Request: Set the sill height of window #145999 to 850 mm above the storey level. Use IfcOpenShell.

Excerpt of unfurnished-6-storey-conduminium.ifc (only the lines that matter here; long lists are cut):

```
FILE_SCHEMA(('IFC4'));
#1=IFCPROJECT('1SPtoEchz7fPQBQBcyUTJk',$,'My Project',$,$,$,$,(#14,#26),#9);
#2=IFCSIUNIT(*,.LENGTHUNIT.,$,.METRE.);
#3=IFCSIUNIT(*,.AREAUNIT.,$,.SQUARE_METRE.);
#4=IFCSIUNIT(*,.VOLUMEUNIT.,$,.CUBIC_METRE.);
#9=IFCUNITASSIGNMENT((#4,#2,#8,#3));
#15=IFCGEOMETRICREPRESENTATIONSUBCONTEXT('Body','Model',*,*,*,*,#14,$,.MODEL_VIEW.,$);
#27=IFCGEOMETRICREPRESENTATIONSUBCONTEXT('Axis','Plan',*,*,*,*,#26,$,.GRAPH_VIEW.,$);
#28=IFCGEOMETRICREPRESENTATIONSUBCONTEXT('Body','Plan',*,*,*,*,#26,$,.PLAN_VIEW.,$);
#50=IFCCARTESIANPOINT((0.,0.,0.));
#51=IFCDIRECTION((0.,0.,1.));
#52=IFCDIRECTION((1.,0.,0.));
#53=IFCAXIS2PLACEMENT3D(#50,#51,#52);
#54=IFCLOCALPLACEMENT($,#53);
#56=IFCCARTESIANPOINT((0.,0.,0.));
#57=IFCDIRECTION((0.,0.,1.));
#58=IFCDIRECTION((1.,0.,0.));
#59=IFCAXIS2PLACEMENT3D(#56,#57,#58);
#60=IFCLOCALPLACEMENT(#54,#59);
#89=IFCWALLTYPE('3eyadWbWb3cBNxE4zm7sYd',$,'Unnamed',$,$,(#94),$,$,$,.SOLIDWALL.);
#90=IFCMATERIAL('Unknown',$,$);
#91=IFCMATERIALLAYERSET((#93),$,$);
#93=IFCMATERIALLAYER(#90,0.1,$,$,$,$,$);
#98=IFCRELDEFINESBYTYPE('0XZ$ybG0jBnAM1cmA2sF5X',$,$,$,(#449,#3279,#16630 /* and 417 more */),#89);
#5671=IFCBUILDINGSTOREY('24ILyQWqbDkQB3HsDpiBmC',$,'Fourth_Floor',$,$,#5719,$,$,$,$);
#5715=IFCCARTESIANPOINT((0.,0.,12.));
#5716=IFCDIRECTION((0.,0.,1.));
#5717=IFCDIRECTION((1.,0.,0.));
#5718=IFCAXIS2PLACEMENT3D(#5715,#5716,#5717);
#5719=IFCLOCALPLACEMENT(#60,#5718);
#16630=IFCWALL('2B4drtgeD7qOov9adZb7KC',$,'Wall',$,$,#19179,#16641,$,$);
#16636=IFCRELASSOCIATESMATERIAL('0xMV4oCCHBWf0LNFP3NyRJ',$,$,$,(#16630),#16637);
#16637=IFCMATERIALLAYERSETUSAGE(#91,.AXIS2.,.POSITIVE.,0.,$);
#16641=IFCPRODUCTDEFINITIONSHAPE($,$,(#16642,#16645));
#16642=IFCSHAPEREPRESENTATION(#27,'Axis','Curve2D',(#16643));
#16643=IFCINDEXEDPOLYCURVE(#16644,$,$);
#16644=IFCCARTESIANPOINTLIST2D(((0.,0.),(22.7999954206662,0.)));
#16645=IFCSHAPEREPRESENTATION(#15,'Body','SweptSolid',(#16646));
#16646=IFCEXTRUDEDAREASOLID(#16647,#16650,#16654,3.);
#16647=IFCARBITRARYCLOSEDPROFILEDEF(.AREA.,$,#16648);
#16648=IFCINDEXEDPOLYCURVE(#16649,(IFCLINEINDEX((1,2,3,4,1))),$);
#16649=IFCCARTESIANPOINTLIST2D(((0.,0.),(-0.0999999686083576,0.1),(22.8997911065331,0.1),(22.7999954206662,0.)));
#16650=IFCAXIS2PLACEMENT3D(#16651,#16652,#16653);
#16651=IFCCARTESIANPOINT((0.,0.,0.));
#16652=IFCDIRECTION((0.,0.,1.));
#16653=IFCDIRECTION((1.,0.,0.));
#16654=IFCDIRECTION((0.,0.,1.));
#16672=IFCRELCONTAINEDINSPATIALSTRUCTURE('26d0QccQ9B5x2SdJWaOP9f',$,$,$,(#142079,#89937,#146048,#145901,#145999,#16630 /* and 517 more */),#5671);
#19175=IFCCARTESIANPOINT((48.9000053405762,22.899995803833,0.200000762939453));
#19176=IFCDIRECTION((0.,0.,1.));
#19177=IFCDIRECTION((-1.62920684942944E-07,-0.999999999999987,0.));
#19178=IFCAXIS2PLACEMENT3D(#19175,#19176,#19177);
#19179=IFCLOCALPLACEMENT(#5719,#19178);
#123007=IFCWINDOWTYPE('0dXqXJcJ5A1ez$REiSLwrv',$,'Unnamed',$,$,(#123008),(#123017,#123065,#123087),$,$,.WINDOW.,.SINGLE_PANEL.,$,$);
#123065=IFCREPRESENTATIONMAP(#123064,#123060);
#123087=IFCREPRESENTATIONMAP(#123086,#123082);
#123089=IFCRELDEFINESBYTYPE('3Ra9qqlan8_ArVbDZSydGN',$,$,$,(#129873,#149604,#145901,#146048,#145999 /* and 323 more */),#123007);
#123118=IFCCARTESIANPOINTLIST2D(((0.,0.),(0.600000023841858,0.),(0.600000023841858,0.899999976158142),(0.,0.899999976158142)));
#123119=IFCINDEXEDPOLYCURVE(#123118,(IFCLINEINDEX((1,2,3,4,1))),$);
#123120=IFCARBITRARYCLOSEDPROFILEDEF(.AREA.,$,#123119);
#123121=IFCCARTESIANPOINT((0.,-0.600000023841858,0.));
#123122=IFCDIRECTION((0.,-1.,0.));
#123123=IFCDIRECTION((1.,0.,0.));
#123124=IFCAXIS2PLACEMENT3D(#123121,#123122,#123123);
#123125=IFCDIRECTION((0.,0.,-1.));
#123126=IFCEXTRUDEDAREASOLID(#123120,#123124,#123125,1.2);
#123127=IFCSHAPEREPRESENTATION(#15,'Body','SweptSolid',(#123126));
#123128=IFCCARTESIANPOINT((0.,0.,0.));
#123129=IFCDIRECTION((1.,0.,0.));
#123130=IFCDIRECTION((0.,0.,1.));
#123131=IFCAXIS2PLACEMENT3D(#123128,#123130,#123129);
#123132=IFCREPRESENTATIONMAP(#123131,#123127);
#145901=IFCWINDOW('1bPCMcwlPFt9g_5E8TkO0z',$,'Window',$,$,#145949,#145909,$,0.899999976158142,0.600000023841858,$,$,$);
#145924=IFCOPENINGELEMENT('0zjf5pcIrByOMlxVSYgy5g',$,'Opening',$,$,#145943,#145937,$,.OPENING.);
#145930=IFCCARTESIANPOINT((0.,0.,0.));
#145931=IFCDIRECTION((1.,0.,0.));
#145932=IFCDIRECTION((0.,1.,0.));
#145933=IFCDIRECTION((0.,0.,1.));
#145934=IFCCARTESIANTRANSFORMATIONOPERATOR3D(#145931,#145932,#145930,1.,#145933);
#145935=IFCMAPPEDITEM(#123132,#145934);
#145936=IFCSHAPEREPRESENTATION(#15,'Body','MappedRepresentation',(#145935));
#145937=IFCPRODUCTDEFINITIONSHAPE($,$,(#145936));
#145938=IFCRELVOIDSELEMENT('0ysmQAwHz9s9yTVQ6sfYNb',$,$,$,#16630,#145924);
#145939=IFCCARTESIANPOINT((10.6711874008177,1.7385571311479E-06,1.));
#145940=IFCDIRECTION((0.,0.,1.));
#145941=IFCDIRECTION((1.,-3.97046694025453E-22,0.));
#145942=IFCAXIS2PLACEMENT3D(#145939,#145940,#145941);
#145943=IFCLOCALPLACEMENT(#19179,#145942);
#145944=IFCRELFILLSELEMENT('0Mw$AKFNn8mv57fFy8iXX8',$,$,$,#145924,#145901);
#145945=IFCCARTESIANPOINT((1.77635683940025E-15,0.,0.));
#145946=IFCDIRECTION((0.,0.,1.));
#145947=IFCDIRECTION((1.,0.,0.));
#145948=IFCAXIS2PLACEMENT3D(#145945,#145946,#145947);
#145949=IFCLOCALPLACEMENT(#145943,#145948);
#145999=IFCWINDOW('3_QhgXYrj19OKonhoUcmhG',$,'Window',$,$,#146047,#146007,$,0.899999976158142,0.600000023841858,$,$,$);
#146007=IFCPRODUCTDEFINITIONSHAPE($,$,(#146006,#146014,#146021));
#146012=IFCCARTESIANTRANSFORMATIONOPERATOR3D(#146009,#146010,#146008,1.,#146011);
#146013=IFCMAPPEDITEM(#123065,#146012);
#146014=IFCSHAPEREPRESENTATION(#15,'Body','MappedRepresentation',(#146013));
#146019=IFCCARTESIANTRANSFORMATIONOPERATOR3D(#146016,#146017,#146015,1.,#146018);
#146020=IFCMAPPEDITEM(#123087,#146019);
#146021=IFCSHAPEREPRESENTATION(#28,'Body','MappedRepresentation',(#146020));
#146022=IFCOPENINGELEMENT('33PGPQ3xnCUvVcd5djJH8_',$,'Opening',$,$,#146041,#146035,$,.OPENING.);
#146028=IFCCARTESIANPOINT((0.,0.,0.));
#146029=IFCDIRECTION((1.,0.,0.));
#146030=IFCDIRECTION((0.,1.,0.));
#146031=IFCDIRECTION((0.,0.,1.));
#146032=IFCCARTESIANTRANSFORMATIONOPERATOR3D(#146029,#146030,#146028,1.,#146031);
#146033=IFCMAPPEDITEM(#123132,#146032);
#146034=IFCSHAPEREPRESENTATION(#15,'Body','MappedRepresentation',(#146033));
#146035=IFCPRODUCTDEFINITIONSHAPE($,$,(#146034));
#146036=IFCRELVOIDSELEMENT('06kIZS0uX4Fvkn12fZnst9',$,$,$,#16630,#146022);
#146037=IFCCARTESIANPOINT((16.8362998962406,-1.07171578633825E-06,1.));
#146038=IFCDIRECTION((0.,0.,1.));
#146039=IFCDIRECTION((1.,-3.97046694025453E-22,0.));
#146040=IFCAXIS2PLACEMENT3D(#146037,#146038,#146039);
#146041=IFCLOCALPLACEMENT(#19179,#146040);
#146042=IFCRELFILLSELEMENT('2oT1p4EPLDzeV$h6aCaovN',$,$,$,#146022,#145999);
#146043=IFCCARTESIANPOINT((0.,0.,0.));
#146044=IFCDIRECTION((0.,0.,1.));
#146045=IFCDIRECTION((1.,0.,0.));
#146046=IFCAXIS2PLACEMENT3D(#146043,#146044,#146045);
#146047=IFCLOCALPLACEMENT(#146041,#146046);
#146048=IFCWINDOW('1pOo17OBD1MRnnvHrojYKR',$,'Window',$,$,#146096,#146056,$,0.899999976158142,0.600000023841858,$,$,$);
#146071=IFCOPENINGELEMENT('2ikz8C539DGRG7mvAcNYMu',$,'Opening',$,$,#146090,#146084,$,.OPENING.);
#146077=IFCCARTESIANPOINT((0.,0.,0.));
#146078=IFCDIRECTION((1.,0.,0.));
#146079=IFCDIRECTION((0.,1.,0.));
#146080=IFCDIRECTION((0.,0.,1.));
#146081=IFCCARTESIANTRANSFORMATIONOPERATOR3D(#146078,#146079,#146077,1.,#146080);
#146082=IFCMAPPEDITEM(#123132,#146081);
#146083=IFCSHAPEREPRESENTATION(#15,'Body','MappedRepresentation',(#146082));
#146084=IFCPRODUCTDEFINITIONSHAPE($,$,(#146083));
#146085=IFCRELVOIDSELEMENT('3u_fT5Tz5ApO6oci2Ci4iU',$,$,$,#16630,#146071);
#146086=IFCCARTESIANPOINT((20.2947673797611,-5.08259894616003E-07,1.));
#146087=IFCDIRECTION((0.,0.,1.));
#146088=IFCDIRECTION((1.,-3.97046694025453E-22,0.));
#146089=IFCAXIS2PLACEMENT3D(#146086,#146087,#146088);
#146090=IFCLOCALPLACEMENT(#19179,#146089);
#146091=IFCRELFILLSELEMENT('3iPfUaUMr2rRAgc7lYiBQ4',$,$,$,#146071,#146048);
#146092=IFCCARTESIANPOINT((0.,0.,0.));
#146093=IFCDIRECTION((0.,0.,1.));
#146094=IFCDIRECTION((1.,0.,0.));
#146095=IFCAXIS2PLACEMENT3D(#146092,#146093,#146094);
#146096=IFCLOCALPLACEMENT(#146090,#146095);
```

```python
import numpy as np
import ifcopenshell
import ifcopenshell.api.geometry
import ifcopenshell.geom
import ifcopenshell.util.element
import ifcopenshell.util.placement
import ifcopenshell.util.shape
import ifcopenshell.util.unit

model = ifcopenshell.open("unfurnished-6-storey-conduminium.ifc")
unit_scale = ifcopenshell.util.unit.calculate_unit_scale(model)

window = model.by_id(145999)
opening = window.FillsVoids[0].RelatingOpeningElement
storey = ifcopenshell.util.element.get_container(window, ifc_class="IfcBuildingStorey")
level = ifcopenshell.util.placement.get_local_placement(storey.ObjectPlacement)[2, 3]

# The opening's origin need not be at the sill, so measure its lowest point.
shape = ifcopenshell.geom.create_shape(ifcopenshell.geom.settings(), opening)
bottom = ifcopenshell.util.shape.get_shape_bottom_elevation(shape, shape.geometry) / unit_scale
dz = level + 0.85 / unit_scale - bottom

shift = np.array([0.0, 0.0, dz])
# The window is placed relative to its opening, so it follows when the opening moves.
matrix = ifcopenshell.util.placement.get_local_placement(opening.ObjectPlacement)
matrix[:3, 3] += shift
ifcopenshell.api.geometry.edit_object_placement(
    model, product=opening, matrix=matrix, is_si=False, should_transform_children=True
)

print(f"moved by {dz * unit_scale:+.3f} m")

model.write("unfurnished-6-storey-conduminium_rev.ifc")
```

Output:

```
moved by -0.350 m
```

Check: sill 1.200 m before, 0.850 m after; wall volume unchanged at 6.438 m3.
